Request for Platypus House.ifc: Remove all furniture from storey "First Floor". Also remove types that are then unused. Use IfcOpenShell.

First a look at what the model holds.

```python
import ifcopenshell
import ifcopenshell.util.element

model = ifcopenshell.open("Platypus House.ifc")
print(model.schema)
storey = next(s for s in model.by_type("IfcBuildingStorey") if s.Name == "First Floor")
furniture = [e for e in ifcopenshell.util.element.get_decomposition(storey) if e.is_a("IfcFurnishingElement")]
seen = {}
for e in furniture:
    element_type = ifcopenshell.util.element.get_type(e)
    name = element_type.Name if element_type not in (None, e) else None
    seen[name] = seen.get(name, 0) + 1
for name, count in sorted(seen.items(), key=str):
    print(count, "x", name)
```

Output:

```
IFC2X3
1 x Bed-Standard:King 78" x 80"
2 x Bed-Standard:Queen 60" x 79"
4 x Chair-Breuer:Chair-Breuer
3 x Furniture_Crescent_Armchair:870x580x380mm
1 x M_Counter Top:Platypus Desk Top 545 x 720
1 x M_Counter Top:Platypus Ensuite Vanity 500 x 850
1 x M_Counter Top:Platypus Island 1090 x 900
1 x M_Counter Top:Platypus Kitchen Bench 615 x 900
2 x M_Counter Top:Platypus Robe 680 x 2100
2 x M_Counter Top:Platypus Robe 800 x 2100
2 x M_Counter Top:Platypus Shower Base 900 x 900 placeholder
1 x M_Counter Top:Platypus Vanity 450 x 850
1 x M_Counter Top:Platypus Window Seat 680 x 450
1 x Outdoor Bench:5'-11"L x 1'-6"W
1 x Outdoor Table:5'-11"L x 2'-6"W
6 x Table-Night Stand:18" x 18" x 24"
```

```python
import ifcopenshell
import ifcopenshell.api.root
import ifcopenshell.util.element

model = ifcopenshell.open("Platypus House.ifc")

storey = next(s for s in model.by_type("IfcBuildingStorey") if s.Name == "First Floor")
furniture = [e for e in ifcopenshell.util.element.get_decomposition(storey) if e.is_a("IfcFurnishingElement")]
types = {ifcopenshell.util.element.get_type(e) for e in furniture} - {None, *furniture}

for e in furniture:
    ifcopenshell.api.root.remove_product(model, product=e)
print(len(furniture), "removed")

unused = [t for t in types if not ifcopenshell.util.element.get_types(t)]
for t in unused:
    ifcopenshell.api.root.remove_product(model, product=t)
print(len(unused), "unused types removed")

model.write("Platypus House-out.ifc")
```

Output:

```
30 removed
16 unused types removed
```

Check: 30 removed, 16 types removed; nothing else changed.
